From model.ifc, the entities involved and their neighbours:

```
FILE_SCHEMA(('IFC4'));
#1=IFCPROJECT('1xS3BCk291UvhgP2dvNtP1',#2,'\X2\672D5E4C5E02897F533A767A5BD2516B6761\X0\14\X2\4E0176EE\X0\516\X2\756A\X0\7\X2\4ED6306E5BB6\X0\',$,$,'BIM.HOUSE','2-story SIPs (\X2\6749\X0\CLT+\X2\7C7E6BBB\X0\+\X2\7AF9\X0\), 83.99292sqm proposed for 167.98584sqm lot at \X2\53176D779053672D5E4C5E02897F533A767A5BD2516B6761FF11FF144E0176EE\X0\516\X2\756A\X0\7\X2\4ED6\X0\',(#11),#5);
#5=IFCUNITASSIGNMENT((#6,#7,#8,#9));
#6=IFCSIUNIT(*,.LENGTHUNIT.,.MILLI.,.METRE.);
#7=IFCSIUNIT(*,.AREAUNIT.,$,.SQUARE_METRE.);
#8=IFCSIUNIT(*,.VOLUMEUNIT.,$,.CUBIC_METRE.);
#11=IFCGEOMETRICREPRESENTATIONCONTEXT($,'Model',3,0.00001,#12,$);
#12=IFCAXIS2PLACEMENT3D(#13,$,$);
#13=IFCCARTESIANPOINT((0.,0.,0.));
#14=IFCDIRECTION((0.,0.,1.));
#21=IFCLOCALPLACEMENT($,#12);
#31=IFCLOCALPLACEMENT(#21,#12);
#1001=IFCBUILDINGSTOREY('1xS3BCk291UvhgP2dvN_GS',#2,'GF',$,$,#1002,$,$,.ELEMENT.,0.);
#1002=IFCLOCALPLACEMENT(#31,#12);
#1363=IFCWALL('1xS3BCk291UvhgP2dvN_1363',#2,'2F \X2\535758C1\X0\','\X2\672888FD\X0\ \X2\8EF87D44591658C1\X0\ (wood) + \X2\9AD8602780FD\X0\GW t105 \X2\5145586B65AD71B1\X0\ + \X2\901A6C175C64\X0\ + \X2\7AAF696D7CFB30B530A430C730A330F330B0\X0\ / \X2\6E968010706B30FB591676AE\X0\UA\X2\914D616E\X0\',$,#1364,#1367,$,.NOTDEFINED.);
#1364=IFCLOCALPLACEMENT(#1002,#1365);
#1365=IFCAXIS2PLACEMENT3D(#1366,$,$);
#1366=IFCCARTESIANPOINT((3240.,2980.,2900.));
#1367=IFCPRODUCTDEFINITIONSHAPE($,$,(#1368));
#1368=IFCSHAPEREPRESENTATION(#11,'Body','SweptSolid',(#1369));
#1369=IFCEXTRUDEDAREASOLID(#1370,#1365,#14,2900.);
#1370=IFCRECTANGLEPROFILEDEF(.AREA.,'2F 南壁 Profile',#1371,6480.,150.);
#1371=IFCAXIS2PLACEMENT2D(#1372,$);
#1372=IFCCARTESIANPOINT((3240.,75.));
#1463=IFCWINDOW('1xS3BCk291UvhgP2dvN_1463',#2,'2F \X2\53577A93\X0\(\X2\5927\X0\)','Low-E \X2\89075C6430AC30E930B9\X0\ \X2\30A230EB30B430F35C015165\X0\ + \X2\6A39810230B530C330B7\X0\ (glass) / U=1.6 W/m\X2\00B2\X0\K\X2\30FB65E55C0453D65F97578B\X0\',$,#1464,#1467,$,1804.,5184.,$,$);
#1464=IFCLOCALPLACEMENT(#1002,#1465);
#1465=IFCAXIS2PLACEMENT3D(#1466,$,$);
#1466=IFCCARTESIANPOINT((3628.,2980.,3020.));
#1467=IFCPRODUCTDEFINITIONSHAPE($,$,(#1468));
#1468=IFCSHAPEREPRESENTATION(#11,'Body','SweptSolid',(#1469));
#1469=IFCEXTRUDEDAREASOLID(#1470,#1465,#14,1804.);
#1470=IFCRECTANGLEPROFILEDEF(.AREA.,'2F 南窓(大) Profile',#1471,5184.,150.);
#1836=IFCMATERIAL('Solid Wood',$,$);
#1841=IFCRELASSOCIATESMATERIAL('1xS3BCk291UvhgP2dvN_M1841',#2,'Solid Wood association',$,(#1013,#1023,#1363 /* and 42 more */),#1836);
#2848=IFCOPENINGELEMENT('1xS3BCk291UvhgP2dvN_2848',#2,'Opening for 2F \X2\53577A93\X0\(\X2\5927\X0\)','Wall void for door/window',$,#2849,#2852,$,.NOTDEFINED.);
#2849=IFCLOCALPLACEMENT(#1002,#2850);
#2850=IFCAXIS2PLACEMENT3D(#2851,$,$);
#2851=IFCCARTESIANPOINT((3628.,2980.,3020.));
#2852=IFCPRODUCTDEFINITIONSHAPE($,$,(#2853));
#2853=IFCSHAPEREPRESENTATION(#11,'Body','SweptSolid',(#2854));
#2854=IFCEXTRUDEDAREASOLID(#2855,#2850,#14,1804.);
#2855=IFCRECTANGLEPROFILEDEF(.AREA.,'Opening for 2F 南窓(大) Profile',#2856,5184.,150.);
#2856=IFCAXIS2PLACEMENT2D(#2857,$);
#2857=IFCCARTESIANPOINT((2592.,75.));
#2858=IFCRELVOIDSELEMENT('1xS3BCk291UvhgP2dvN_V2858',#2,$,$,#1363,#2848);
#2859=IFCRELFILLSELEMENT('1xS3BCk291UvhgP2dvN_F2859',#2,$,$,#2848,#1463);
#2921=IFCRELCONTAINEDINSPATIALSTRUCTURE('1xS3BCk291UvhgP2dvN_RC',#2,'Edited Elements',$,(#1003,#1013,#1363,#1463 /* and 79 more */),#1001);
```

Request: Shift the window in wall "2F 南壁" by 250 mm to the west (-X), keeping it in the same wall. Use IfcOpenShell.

```python
import ifcopenshell
import ifcopenshell.api.geometry
import ifcopenshell.util.placement
import ifcopenshell.util.unit

model = ifcopenshell.open("model.ifc")
unit_scale = ifcopenshell.util.unit.calculate_unit_scale(model)

window = model.by_id(1463)
opening = window.FillsVoids[0].RelatingOpeningElement
wall = opening.VoidsElements[0].RelatingBuildingElement

wall_matrix = ifcopenshell.util.placement.get_local_placement(wall.ObjectPlacement)
shift = wall_matrix[:3, 0] * -0.25 / unit_scale
before = ifcopenshell.util.placement.get_local_placement(window.ObjectPlacement)[:3, 3].copy()

# The window is not placed relative to its opening, so move both.
for product in (opening, window):
    matrix = ifcopenshell.util.placement.get_local_placement(product.ObjectPlacement)
    matrix[:3, 3] += shift
    ifcopenshell.api.geometry.edit_object_placement(model, product=product, matrix=matrix, is_si=False)

after = ifcopenshell.util.placement.get_local_placement(window.ObjectPlacement)[:3, 3]
print("window moved by", (after - before).round(3) + 0.0)

model.write("model-out.ifc")
```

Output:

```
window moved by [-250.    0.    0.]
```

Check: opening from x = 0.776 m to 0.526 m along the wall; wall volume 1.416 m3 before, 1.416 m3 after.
